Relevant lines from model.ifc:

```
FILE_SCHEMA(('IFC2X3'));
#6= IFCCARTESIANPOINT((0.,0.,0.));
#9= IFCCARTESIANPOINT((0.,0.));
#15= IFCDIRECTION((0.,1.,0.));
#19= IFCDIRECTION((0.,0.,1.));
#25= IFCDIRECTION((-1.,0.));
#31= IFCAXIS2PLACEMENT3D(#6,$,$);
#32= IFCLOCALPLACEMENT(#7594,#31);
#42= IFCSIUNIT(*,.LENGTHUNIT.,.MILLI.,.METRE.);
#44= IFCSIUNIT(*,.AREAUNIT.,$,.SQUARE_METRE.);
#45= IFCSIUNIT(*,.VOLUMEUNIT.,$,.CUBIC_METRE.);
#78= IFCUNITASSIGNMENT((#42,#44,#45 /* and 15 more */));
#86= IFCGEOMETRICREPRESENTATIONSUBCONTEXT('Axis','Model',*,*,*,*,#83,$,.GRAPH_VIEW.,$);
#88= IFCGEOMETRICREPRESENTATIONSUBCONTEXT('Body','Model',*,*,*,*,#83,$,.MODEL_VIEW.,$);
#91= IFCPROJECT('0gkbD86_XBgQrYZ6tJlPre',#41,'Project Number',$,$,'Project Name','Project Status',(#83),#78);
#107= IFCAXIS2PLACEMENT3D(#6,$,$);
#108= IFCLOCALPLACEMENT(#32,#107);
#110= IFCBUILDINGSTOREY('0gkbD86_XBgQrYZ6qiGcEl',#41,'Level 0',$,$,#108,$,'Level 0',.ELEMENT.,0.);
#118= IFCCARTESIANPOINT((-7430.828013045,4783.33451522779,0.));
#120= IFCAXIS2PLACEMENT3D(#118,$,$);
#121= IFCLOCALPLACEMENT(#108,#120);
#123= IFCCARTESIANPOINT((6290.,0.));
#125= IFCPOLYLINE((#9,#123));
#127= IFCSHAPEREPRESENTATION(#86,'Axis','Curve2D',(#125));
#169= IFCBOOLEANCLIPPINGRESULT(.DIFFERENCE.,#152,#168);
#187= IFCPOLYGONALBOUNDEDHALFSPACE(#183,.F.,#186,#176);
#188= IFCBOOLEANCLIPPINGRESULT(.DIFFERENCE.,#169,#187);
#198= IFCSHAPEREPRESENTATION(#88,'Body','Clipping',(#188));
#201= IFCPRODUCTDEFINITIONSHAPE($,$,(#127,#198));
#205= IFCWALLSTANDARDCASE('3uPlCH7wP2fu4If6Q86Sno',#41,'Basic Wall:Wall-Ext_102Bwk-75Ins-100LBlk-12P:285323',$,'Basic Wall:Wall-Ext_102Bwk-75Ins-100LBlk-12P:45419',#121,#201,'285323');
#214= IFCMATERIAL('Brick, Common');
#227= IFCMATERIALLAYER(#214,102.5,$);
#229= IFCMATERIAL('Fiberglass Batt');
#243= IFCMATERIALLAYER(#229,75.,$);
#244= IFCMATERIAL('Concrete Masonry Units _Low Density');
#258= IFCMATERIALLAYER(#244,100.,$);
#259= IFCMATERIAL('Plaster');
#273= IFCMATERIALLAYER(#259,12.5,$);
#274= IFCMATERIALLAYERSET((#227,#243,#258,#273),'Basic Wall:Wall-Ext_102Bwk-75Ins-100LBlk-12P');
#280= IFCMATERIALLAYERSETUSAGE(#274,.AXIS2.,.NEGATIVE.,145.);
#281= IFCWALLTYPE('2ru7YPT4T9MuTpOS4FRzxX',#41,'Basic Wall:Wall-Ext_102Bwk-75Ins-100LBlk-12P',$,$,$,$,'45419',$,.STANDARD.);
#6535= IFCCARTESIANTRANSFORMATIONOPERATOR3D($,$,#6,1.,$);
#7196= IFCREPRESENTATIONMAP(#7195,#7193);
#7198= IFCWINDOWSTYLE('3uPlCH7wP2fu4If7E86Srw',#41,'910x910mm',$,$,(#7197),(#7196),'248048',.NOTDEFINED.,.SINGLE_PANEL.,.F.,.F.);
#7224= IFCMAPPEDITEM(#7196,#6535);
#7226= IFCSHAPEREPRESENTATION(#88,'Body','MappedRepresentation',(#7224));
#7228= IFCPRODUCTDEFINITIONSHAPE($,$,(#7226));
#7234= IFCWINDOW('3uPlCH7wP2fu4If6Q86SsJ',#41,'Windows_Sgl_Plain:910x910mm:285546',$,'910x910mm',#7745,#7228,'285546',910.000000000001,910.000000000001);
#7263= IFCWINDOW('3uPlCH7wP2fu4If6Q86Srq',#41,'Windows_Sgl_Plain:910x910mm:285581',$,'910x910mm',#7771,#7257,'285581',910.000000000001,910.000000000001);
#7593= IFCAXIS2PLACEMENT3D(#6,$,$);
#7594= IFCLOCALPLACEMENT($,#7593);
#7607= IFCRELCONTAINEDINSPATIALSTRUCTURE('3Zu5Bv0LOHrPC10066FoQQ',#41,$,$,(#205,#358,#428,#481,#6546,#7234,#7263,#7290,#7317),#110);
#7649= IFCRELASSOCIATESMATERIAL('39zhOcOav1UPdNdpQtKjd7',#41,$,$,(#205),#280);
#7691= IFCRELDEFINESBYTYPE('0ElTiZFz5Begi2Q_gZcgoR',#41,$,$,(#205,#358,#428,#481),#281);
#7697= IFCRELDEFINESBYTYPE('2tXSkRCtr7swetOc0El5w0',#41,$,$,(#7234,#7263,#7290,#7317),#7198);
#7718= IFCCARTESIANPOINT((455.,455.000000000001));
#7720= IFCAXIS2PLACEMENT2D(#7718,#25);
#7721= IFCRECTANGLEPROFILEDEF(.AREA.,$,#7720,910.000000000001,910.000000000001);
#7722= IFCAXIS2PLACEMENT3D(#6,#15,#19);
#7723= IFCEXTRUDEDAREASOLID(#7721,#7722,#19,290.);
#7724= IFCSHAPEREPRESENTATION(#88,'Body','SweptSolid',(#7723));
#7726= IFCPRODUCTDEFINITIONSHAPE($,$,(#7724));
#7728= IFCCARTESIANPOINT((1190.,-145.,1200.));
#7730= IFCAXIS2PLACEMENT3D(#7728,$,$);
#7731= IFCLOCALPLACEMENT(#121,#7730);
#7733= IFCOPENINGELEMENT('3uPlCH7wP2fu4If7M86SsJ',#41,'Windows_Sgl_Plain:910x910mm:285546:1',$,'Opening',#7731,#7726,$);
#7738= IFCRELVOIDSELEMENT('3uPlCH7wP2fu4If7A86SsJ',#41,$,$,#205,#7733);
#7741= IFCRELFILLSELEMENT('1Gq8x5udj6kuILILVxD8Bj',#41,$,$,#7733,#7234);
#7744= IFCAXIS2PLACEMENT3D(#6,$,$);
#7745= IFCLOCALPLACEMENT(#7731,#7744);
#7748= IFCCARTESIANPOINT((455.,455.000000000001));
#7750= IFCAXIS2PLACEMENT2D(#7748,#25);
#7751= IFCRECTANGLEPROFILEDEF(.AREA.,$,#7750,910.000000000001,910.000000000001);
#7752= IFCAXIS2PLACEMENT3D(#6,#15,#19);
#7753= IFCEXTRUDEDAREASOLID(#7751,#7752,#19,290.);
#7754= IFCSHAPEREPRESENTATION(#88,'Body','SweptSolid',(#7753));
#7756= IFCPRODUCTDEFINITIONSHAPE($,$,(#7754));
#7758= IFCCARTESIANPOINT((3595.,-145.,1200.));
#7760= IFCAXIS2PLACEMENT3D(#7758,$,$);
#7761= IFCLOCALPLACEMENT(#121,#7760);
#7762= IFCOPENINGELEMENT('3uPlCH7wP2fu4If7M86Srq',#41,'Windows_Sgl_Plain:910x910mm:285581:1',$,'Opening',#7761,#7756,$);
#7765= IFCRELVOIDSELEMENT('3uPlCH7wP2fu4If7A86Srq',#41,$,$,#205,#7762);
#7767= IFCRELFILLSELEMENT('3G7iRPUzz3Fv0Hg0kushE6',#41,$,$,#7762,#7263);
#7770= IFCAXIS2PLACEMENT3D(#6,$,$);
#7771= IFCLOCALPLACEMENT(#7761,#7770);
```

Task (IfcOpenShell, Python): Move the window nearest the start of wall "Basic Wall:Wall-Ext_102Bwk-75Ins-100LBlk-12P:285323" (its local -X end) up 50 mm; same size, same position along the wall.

```python
import numpy as np
import ifcopenshell
import ifcopenshell.api.geometry
import ifcopenshell.util.placement
import ifcopenshell.util.unit

model = ifcopenshell.open("model.ifc")
unit_scale = ifcopenshell.util.unit.calculate_unit_scale(model)

window = model.by_id(7234)
opening = window.FillsVoids[0].RelatingOpeningElement
dz = 0.05 / unit_scale

shift = np.array([0.0, 0.0, dz])
# The window is placed relative to its opening, so it follows when the opening moves.
matrix = ifcopenshell.util.placement.get_local_placement(opening.ObjectPlacement)
matrix[:3, 3] += shift
ifcopenshell.api.geometry.edit_object_placement(
    model, product=opening, matrix=matrix, is_si=False, should_transform_children=True
)

print(f"moved by {dz * unit_scale:+.3f} m")

model.write("model_v2.ifc")
```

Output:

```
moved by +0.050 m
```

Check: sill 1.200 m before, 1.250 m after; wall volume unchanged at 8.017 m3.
